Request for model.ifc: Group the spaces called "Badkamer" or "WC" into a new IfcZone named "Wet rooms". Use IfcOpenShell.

First a look at what the model holds.

```python
import ifcopenshell

model = ifcopenshell.open("model.ifc")
print(model.schema)
seen = {}
for space in model.by_type("IfcSpace"):
    seen[space.LongName] = seen.get(space.LongName, 0) + 1
for name, count in sorted(seen.items(), key=str):
    print(count, "x", name)
print("zones:", [z.Name for z in model.by_type("IfcZone")][:20])
```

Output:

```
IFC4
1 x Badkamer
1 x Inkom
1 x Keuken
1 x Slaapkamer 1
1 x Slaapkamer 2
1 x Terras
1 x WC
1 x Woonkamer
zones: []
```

```python
import ifcopenshell
import ifcopenshell.api.group
import ifcopenshell.api.root

model = ifcopenshell.open("model.ifc")

names = {"Badkamer", "WC"}
spaces = [s for s in model.by_type("IfcSpace") if s.LongName in names]

zone = ifcopenshell.api.root.create_entity(model, ifc_class="IfcZone", name="Wet rooms")
ifcopenshell.api.group.assign_group(model, products=spaces, group=zone)
print(len(spaces), "spaces in", zone.Name)

model.write("model_rev.ifc")
```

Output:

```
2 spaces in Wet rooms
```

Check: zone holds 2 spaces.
